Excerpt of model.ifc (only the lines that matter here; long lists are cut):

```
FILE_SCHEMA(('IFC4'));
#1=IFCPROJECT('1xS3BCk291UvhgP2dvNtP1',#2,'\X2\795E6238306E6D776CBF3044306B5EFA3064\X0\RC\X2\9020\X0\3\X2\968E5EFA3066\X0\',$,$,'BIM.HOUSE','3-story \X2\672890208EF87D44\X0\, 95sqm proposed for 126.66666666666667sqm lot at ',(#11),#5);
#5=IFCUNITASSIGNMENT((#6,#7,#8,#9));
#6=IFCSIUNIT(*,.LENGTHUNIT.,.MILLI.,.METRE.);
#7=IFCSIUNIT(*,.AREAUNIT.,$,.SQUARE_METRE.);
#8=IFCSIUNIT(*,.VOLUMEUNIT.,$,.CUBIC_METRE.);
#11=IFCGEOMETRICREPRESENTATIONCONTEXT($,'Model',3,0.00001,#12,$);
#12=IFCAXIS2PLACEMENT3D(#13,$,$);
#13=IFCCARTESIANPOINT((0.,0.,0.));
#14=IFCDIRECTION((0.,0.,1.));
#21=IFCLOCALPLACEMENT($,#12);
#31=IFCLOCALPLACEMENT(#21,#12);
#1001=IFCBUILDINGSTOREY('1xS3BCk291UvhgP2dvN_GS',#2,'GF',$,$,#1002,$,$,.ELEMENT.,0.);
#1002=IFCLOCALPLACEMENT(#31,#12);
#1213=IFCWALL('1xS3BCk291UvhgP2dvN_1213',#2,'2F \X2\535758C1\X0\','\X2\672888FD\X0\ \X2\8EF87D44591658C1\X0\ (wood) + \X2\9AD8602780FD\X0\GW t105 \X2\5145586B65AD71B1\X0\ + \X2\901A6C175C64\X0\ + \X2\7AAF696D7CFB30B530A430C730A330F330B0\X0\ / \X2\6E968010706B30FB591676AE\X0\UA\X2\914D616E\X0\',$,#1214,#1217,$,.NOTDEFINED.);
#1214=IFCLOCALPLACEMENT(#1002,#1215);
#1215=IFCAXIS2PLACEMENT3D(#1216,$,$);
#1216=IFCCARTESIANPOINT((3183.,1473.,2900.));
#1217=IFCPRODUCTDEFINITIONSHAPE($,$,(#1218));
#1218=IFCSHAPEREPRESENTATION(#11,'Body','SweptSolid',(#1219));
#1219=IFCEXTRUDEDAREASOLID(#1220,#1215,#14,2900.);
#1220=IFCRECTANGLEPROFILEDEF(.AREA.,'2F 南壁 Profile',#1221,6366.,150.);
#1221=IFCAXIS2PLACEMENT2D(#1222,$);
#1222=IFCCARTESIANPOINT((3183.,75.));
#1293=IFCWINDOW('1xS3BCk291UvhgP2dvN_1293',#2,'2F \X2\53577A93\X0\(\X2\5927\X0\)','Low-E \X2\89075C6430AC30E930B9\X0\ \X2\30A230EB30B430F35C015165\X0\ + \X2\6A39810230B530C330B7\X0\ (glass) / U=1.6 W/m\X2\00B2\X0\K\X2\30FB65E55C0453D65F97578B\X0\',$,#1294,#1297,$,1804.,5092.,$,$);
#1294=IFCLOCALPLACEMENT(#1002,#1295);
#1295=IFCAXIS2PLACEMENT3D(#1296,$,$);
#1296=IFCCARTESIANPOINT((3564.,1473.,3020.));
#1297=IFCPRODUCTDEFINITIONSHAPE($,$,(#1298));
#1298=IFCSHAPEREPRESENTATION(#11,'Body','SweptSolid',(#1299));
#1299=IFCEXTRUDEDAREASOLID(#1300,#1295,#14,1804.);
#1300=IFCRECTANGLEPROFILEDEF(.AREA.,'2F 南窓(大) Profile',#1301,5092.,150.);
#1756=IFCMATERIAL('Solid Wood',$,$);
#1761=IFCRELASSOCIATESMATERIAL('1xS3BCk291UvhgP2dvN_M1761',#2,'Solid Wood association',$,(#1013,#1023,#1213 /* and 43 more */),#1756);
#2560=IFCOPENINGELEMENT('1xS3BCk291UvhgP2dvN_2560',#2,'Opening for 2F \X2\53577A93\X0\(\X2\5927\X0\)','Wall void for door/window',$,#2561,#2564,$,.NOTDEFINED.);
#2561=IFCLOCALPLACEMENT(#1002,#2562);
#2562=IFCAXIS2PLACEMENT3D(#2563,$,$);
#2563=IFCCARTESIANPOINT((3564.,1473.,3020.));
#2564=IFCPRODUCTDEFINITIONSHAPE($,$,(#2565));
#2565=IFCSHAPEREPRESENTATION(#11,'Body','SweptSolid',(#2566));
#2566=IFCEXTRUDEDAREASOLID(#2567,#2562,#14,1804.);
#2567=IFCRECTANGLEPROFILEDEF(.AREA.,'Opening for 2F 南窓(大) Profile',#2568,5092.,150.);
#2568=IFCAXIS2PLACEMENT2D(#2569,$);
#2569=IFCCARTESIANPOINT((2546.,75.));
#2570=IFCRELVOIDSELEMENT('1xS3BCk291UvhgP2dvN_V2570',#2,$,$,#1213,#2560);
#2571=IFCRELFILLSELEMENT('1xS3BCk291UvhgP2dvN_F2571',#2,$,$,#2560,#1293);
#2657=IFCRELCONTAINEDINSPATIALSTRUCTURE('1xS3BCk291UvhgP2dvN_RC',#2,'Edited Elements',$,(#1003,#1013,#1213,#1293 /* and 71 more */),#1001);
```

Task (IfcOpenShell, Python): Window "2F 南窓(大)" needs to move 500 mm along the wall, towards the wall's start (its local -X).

```python
import ifcopenshell
import ifcopenshell.api.geometry
import ifcopenshell.util.placement
import ifcopenshell.util.unit

model = ifcopenshell.open("model.ifc")
unit_scale = ifcopenshell.util.unit.calculate_unit_scale(model)

window = model.by_guid("1xS3BCk291UvhgP2dvN_1293")
opening = window.FillsVoids[0].RelatingOpeningElement
wall = opening.VoidsElements[0].RelatingBuildingElement

wall_matrix = ifcopenshell.util.placement.get_local_placement(wall.ObjectPlacement)
shift = wall_matrix[:3, 0] * -0.5 / unit_scale
before = ifcopenshell.util.placement.get_local_placement(window.ObjectPlacement)[:3, 3].copy()

# The window is not placed relative to its opening, so move both.
for product in (opening, window):
    matrix = ifcopenshell.util.placement.get_local_placement(product.ObjectPlacement)
    matrix[:3, 3] += shift
    ifcopenshell.api.geometry.edit_object_placement(model, product=product, matrix=matrix, is_si=False)

after = ifcopenshell.util.placement.get_local_placement(window.ObjectPlacement)[:3, 3]
print("window moved by", (after - before).round(3) + 0.0)

model.write("model_v2.ifc")
```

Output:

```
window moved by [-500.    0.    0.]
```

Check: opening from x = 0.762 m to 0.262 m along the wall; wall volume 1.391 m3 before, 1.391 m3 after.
